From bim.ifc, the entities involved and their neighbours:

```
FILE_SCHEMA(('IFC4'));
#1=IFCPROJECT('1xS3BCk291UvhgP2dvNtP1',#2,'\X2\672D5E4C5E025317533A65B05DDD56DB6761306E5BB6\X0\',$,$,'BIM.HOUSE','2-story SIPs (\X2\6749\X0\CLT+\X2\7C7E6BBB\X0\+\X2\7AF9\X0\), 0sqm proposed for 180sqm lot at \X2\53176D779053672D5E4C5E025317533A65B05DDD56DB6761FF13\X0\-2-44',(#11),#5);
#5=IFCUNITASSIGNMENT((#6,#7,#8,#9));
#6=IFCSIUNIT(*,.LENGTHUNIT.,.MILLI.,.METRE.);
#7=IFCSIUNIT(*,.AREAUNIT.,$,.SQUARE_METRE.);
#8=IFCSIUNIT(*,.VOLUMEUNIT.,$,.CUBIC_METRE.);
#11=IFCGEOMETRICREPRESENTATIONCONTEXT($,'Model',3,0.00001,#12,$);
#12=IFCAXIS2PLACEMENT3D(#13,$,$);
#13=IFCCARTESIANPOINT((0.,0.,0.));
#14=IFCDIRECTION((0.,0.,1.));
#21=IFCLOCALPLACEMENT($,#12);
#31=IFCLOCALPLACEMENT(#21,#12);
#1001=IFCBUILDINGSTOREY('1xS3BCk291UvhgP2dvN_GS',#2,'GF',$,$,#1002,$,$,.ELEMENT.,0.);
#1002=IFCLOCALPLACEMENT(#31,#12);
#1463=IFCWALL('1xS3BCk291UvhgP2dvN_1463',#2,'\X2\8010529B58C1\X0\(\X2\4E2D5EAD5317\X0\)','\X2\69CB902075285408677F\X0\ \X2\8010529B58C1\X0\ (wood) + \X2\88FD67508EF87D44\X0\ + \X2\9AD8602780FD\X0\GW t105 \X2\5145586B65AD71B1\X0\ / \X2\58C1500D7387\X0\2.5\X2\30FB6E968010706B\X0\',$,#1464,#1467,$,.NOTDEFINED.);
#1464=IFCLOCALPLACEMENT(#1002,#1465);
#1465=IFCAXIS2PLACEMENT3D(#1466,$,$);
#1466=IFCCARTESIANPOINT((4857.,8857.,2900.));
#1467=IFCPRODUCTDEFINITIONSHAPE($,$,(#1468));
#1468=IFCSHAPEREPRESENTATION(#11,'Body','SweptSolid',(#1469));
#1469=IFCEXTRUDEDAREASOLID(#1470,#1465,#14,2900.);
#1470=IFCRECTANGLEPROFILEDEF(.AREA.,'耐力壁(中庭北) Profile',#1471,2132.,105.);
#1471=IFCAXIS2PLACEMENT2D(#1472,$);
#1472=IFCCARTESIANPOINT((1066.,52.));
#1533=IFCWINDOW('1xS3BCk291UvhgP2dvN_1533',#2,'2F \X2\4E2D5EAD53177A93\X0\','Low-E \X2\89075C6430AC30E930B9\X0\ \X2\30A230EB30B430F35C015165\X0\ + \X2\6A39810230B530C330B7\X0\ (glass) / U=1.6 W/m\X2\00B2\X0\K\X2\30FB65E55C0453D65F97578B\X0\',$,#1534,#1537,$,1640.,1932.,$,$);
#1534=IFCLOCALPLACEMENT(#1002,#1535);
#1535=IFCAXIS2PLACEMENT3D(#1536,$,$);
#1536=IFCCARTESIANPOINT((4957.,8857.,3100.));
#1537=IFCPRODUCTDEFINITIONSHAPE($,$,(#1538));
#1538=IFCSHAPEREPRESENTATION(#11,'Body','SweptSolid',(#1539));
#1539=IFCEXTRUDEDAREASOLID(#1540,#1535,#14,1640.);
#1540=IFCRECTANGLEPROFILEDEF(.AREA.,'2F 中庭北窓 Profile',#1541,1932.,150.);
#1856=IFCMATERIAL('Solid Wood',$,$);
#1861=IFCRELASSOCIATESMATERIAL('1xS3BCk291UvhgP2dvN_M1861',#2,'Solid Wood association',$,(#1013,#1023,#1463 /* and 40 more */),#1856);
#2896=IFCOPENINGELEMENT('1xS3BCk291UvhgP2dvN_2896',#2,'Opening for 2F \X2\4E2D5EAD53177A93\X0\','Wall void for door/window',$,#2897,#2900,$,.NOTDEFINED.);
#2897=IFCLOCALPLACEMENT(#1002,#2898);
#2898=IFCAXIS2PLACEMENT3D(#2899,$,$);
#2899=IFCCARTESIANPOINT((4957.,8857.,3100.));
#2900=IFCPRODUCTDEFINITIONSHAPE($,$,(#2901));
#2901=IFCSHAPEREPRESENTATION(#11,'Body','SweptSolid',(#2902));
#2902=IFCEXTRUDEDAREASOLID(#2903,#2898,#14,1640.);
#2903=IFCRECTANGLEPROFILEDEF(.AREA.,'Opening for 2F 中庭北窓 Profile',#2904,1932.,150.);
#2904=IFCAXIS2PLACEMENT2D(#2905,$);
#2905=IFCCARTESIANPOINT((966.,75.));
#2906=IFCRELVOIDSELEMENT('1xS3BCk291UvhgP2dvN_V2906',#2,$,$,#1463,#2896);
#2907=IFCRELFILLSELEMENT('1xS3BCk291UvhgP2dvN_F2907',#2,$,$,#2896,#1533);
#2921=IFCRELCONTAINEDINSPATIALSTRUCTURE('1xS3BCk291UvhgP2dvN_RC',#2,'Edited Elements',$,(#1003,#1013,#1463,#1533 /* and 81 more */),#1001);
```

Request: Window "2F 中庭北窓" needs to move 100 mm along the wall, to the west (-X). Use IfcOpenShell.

```python
import ifcopenshell
import ifcopenshell.api.geometry
import ifcopenshell.util.placement
import ifcopenshell.util.unit

model = ifcopenshell.open("bim.ifc")
unit_scale = ifcopenshell.util.unit.calculate_unit_scale(model)

window = model.by_guid("1xS3BCk291UvhgP2dvN_1533")
opening = window.FillsVoids[0].RelatingOpeningElement
wall = opening.VoidsElements[0].RelatingBuildingElement

wall_matrix = ifcopenshell.util.placement.get_local_placement(wall.ObjectPlacement)
shift = wall_matrix[:3, 0] * -0.1 / unit_scale
before = ifcopenshell.util.placement.get_local_placement(window.ObjectPlacement)[:3, 3].copy()

# The window is not placed relative to its opening, so move both.
for product in (opening, window):
    matrix = ifcopenshell.util.placement.get_local_placement(product.ObjectPlacement)
    matrix[:3, 3] += shift
    ifcopenshell.api.geometry.edit_object_placement(model, product=product, matrix=matrix, is_si=False)

after = ifcopenshell.util.placement.get_local_placement(window.ObjectPlacement)[:3, 3]
print("window moved by", (after - before).round(3) + 0.0)

model.write("bim_updated.ifc")
```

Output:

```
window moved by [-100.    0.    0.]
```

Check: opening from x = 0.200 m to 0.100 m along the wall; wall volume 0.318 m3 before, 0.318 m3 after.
